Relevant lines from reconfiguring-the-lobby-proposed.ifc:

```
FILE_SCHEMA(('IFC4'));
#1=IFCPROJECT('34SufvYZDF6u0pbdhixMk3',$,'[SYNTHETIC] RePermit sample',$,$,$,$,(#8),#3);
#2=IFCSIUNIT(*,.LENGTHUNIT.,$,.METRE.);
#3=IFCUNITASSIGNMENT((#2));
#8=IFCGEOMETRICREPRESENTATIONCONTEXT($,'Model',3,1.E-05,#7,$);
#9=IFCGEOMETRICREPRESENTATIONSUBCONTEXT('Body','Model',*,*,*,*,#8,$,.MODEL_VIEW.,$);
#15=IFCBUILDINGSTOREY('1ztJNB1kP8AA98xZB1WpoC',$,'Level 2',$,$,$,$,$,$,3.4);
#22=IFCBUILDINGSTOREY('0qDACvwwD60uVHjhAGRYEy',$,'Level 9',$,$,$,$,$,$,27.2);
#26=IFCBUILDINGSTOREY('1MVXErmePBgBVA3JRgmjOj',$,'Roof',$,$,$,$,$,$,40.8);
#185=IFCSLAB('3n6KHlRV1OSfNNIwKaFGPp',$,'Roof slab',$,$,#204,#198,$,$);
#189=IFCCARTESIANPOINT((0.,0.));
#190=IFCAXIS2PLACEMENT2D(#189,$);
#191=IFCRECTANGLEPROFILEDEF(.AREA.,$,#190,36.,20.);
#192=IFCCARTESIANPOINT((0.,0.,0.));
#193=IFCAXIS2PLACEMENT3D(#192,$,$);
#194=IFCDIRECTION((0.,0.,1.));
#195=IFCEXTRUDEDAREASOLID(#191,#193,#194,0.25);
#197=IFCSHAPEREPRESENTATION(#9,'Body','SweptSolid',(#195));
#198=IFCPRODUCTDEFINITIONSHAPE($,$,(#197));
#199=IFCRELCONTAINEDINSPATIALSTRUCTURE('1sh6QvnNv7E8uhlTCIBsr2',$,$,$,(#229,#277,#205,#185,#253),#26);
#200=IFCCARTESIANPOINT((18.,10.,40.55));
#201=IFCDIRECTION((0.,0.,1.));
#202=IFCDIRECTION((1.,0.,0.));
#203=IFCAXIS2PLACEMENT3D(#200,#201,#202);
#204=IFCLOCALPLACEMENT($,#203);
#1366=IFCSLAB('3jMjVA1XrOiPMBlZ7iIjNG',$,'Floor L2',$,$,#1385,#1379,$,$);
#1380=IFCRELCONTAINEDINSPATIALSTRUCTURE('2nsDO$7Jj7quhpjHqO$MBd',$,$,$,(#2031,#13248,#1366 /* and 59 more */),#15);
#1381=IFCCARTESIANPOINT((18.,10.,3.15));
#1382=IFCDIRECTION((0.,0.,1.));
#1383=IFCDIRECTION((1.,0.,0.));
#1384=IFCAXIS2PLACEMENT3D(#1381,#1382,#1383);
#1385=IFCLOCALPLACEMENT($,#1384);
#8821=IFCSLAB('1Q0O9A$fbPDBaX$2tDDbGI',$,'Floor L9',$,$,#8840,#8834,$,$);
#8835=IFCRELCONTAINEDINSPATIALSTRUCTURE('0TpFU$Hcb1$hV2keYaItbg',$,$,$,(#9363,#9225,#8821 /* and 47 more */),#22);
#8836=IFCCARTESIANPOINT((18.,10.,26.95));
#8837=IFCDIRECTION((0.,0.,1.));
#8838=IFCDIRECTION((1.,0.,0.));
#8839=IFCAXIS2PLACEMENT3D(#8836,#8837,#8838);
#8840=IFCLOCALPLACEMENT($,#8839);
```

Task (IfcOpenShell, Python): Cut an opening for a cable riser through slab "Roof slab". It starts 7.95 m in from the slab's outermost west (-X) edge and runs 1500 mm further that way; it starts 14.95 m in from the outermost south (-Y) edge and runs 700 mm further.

```python
import numpy as np
import ifcopenshell
import ifcopenshell.api.feature
import ifcopenshell.api.geometry
import ifcopenshell.api.root
import ifcopenshell.geom
import ifcopenshell.util.placement
import ifcopenshell.util.representation
import ifcopenshell.util.shape
import ifcopenshell.util.unit

model = ifcopenshell.open("reconfiguring-the-lobby-proposed.ifc")
unit_scale = ifcopenshell.util.unit.calculate_unit_scale(model)
settings = ifcopenshell.geom.settings()


def volume(element):
    """Net volume in cubic metres, openings subtracted."""
    shape = ifcopenshell.geom.create_shape(settings, element)
    return ifcopenshell.util.shape.get_volume(shape.geometry)


slab = model.by_guid("3n6KHlRV1OSfNNIwKaFGPp")
before = volume(slab)

# Extent in the slab's own axes, in metres. The edges named are its -X and -Y sides.
slab_shape = ifcopenshell.geom.create_shape(settings, slab)
vertices = ifcopenshell.util.shape.get_vertices(slab_shape.geometry)
x_min, y_min, bottom = vertices.min(axis=0)
top = vertices[:, 2].max()

opening = ifcopenshell.api.root.create_entity(model, ifc_class="IfcOpeningElement", name="Cable riser opening", predefined_type="OPENING")
context = ifcopenshell.util.representation.get_context(model, "Model", "Body", "MODEL_VIEW")
width, depth = 1.5, 0.7
outline = [(0.0, 0.0), (width, 0.0), (width, depth), (0.0, depth), (0.0, 0.0)]
# Overshoot both faces by 50 mm so the cut is clean.
shape = ifcopenshell.api.geometry.add_slab_representation(
    model, context=context, depth=top - bottom + 0.1, polyline=outline
)
ifcopenshell.api.geometry.assign_representation(model, product=opening, representation=shape)

matrix = ifcopenshell.util.placement.get_local_placement(slab.ObjectPlacement)
matrix[:, 3] = matrix @ np.append(np.array([x_min + 7.95, y_min + 14.95, bottom - 0.05]) / unit_scale, 1.0)
ifcopenshell.api.geometry.edit_object_placement(model, product=opening, matrix=matrix, is_si=False)
ifcopenshell.api.feature.add_feature(model, feature=opening, element=slab)

after = volume(slab)

print(f"slab volume {before:.3f} -> {after:.3f} m3")

model.write("reconfiguring-the-lobby-proposed_updated.ifc")
```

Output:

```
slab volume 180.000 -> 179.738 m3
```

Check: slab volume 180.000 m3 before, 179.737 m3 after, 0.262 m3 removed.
